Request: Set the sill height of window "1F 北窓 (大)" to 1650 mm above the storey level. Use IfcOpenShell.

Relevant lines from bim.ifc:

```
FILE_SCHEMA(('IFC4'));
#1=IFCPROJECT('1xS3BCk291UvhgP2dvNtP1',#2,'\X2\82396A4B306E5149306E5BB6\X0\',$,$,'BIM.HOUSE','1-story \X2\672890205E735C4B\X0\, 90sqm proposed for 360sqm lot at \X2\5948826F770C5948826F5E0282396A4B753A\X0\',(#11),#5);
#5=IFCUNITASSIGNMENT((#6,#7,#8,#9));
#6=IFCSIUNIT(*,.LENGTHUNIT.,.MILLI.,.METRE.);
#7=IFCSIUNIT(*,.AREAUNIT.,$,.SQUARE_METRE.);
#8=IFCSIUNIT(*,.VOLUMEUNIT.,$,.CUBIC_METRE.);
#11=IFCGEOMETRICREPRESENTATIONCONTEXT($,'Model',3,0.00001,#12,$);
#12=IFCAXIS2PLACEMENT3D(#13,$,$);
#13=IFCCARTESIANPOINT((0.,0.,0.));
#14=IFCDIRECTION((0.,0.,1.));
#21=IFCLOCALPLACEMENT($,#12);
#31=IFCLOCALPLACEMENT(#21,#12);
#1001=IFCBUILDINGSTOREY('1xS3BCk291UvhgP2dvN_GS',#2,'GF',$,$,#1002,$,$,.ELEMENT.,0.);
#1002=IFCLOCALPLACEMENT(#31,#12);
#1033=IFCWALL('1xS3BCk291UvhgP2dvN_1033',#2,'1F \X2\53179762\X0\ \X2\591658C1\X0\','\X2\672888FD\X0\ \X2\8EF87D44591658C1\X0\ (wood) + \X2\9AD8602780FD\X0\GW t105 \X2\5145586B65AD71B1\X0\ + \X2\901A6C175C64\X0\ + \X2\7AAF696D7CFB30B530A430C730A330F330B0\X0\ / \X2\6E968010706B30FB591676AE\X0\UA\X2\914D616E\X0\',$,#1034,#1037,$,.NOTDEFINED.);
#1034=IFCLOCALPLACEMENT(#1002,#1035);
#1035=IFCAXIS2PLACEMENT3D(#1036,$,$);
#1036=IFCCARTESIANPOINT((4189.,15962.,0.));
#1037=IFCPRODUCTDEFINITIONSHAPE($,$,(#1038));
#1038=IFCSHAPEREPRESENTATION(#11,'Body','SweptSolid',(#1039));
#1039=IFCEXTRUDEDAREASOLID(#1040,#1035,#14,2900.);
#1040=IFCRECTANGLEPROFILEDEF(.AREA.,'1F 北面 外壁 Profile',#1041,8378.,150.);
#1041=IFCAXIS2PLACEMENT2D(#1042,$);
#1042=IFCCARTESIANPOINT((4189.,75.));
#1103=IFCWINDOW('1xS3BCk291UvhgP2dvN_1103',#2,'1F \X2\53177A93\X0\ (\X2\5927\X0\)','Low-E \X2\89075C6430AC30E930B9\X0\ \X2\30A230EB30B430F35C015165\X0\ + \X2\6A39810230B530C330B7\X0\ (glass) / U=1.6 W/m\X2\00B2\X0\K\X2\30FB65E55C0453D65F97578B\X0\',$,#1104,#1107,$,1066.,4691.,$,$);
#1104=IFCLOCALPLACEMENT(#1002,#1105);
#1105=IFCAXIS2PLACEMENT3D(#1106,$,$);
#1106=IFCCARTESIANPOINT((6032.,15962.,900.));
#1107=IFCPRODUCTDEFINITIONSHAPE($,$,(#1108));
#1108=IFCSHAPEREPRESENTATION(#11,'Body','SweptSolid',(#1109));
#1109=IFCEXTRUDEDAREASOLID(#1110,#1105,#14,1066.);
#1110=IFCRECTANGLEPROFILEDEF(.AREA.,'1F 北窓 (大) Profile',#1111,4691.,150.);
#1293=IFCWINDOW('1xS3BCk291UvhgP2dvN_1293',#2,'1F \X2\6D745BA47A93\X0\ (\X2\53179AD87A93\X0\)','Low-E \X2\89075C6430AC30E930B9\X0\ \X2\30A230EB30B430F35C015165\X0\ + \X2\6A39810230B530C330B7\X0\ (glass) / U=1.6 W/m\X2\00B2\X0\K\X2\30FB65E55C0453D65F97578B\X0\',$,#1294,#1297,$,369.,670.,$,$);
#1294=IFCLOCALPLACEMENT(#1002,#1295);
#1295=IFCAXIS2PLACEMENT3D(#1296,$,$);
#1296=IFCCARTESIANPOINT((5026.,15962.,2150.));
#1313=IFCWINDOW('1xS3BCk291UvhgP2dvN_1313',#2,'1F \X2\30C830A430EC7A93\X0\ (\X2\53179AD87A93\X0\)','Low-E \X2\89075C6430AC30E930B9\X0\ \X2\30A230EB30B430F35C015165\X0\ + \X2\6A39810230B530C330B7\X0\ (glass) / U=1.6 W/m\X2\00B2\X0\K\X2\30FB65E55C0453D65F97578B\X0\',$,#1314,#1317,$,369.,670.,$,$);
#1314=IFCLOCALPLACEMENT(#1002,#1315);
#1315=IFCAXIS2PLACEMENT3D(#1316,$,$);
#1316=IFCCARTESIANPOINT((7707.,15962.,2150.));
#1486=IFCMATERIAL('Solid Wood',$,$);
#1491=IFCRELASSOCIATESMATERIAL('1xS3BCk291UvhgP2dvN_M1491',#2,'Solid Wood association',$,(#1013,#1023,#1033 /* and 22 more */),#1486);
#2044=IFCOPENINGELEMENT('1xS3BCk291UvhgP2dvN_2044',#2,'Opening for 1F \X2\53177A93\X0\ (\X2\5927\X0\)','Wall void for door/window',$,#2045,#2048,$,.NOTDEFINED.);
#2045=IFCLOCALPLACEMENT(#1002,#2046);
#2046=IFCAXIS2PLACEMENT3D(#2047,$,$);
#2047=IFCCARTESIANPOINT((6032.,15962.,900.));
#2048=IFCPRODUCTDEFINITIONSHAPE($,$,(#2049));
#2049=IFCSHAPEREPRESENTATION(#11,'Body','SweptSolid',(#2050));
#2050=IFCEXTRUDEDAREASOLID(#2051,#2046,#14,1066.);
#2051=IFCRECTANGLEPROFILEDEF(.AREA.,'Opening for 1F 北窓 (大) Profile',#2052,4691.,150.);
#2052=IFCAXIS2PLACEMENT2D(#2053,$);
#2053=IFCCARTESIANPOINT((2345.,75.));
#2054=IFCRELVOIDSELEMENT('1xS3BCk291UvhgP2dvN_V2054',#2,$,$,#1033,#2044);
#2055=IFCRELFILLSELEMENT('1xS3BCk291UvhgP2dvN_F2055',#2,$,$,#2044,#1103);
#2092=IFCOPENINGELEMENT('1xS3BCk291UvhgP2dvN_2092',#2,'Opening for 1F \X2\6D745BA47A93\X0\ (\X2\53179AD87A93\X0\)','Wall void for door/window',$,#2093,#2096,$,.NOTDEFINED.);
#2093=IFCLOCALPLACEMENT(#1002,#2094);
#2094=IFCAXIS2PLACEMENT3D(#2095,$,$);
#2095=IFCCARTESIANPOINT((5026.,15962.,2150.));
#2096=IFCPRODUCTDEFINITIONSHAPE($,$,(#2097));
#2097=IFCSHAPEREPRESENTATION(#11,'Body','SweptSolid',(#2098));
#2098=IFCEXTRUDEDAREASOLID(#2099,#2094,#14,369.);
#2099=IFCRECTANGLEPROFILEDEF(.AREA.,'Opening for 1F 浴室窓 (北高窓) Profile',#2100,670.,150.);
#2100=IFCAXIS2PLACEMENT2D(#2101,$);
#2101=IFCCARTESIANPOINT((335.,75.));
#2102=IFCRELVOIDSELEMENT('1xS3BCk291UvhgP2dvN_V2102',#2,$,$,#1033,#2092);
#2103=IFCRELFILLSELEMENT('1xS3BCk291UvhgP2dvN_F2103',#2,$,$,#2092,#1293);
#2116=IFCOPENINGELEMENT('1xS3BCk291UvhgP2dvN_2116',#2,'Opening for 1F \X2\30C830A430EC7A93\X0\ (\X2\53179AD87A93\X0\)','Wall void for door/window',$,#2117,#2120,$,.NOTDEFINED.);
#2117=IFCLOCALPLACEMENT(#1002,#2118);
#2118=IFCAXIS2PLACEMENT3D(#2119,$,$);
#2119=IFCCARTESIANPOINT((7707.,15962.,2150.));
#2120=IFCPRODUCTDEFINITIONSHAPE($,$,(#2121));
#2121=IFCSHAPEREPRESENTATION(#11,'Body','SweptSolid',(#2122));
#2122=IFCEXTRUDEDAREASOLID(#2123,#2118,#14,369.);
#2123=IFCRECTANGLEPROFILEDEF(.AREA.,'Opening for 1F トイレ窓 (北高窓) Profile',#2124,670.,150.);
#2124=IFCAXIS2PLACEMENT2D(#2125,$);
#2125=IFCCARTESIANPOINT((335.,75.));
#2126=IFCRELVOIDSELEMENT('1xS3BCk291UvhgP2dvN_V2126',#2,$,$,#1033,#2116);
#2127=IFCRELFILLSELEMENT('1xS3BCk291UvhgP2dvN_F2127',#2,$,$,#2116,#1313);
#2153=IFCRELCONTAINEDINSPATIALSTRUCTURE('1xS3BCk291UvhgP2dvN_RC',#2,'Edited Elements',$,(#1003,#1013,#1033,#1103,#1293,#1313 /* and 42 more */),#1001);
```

```python
import numpy as np
import ifcopenshell
import ifcopenshell.api.geometry
import ifcopenshell.geom
import ifcopenshell.util.element
import ifcopenshell.util.placement
import ifcopenshell.util.shape
import ifcopenshell.util.unit

model = ifcopenshell.open("bim.ifc")
unit_scale = ifcopenshell.util.unit.calculate_unit_scale(model)

window = model.by_id(1103)
opening = window.FillsVoids[0].RelatingOpeningElement
storey = ifcopenshell.util.element.get_container(window, ifc_class="IfcBuildingStorey")
level = ifcopenshell.util.placement.get_local_placement(storey.ObjectPlacement)[2, 3]

# The opening's origin need not be at the sill, so measure its lowest point.
shape = ifcopenshell.geom.create_shape(ifcopenshell.geom.settings(), opening)
bottom = ifcopenshell.util.shape.get_shape_bottom_elevation(shape, shape.geometry) / unit_scale
dz = level + 1.65 / unit_scale - bottom

shift = np.array([0.0, 0.0, dz])
# The window is not placed relative to its opening, so move both.
for product in (opening, window):
    matrix = ifcopenshell.util.placement.get_local_placement(product.ObjectPlacement)
    matrix[:3, 3] += shift
    ifcopenshell.api.geometry.edit_object_placement(model, product=product, matrix=matrix, is_si=False)

print(f"moved by {dz * unit_scale:+.3f} m")

model.write("bim_edited.ifc")
```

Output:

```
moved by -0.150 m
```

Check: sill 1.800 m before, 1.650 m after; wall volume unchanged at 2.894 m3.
